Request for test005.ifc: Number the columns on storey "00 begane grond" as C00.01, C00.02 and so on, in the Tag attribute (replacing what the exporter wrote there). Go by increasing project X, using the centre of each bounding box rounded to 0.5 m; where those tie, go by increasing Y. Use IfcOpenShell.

First a look at what the model holds.

```python
import ifcopenshell
import ifcopenshell.util.element
import ifcopenshell.util.placement

model = ifcopenshell.open("test005.ifc")
print(model.schema)
storey = next(s for s in model.by_type("IfcBuildingStorey") if s.Name == "00 begane grond")
columns = [e for e in ifcopenshell.util.element.get_decomposition(storey) if e.is_a("IfcColumn")]
for e in sorted(columns, key=lambda e: e.id()):
    origin = ifcopenshell.util.placement.get_local_placement(e.ObjectPlacement)[:3, 3]
    print(e.id(), e.Tag, e.Name, origin.round(2) + 0.0, sep=" | ")
```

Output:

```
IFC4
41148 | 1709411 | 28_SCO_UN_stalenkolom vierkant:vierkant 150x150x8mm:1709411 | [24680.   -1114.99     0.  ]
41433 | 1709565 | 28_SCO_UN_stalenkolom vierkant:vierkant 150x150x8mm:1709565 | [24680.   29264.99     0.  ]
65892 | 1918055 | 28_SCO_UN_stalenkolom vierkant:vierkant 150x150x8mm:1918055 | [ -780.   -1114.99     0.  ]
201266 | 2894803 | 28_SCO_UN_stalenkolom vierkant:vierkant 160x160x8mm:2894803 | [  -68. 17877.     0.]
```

```python
import ifcopenshell
import ifcopenshell.geom
import ifcopenshell.util.element
import ifcopenshell.util.shape

model = ifcopenshell.open("test005.ifc")
settings = ifcopenshell.geom.settings()
settings.set("use-world-coords", True)


def centre(element):
    shape = ifcopenshell.geom.create_shape(settings, element)
    return ifcopenshell.util.shape.get_bbox_centroid(shape.geometry)


storey = next(s for s in model.by_type("IfcBuildingStorey") if s.Name == "00 begane grond")
columns = [e for e in ifcopenshell.util.element.get_decomposition(storey) if e.is_a("IfcColumn")]

# Insertion points can sit at a corner or the storey origin, so sort by the geometry (in metres).
centres = {e: centre(e) for e in columns}
columns.sort(key=lambda e: (round(centres[e][0] / 0.5), centres[e][1]))

for i, e in enumerate(columns, start=1):
    number = f"C00.{i:02d}"
    e.Tag = number
    print(e.id(), number)

model.write("test005-out.ifc")
```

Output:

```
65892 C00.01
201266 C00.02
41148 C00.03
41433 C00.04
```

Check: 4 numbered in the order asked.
